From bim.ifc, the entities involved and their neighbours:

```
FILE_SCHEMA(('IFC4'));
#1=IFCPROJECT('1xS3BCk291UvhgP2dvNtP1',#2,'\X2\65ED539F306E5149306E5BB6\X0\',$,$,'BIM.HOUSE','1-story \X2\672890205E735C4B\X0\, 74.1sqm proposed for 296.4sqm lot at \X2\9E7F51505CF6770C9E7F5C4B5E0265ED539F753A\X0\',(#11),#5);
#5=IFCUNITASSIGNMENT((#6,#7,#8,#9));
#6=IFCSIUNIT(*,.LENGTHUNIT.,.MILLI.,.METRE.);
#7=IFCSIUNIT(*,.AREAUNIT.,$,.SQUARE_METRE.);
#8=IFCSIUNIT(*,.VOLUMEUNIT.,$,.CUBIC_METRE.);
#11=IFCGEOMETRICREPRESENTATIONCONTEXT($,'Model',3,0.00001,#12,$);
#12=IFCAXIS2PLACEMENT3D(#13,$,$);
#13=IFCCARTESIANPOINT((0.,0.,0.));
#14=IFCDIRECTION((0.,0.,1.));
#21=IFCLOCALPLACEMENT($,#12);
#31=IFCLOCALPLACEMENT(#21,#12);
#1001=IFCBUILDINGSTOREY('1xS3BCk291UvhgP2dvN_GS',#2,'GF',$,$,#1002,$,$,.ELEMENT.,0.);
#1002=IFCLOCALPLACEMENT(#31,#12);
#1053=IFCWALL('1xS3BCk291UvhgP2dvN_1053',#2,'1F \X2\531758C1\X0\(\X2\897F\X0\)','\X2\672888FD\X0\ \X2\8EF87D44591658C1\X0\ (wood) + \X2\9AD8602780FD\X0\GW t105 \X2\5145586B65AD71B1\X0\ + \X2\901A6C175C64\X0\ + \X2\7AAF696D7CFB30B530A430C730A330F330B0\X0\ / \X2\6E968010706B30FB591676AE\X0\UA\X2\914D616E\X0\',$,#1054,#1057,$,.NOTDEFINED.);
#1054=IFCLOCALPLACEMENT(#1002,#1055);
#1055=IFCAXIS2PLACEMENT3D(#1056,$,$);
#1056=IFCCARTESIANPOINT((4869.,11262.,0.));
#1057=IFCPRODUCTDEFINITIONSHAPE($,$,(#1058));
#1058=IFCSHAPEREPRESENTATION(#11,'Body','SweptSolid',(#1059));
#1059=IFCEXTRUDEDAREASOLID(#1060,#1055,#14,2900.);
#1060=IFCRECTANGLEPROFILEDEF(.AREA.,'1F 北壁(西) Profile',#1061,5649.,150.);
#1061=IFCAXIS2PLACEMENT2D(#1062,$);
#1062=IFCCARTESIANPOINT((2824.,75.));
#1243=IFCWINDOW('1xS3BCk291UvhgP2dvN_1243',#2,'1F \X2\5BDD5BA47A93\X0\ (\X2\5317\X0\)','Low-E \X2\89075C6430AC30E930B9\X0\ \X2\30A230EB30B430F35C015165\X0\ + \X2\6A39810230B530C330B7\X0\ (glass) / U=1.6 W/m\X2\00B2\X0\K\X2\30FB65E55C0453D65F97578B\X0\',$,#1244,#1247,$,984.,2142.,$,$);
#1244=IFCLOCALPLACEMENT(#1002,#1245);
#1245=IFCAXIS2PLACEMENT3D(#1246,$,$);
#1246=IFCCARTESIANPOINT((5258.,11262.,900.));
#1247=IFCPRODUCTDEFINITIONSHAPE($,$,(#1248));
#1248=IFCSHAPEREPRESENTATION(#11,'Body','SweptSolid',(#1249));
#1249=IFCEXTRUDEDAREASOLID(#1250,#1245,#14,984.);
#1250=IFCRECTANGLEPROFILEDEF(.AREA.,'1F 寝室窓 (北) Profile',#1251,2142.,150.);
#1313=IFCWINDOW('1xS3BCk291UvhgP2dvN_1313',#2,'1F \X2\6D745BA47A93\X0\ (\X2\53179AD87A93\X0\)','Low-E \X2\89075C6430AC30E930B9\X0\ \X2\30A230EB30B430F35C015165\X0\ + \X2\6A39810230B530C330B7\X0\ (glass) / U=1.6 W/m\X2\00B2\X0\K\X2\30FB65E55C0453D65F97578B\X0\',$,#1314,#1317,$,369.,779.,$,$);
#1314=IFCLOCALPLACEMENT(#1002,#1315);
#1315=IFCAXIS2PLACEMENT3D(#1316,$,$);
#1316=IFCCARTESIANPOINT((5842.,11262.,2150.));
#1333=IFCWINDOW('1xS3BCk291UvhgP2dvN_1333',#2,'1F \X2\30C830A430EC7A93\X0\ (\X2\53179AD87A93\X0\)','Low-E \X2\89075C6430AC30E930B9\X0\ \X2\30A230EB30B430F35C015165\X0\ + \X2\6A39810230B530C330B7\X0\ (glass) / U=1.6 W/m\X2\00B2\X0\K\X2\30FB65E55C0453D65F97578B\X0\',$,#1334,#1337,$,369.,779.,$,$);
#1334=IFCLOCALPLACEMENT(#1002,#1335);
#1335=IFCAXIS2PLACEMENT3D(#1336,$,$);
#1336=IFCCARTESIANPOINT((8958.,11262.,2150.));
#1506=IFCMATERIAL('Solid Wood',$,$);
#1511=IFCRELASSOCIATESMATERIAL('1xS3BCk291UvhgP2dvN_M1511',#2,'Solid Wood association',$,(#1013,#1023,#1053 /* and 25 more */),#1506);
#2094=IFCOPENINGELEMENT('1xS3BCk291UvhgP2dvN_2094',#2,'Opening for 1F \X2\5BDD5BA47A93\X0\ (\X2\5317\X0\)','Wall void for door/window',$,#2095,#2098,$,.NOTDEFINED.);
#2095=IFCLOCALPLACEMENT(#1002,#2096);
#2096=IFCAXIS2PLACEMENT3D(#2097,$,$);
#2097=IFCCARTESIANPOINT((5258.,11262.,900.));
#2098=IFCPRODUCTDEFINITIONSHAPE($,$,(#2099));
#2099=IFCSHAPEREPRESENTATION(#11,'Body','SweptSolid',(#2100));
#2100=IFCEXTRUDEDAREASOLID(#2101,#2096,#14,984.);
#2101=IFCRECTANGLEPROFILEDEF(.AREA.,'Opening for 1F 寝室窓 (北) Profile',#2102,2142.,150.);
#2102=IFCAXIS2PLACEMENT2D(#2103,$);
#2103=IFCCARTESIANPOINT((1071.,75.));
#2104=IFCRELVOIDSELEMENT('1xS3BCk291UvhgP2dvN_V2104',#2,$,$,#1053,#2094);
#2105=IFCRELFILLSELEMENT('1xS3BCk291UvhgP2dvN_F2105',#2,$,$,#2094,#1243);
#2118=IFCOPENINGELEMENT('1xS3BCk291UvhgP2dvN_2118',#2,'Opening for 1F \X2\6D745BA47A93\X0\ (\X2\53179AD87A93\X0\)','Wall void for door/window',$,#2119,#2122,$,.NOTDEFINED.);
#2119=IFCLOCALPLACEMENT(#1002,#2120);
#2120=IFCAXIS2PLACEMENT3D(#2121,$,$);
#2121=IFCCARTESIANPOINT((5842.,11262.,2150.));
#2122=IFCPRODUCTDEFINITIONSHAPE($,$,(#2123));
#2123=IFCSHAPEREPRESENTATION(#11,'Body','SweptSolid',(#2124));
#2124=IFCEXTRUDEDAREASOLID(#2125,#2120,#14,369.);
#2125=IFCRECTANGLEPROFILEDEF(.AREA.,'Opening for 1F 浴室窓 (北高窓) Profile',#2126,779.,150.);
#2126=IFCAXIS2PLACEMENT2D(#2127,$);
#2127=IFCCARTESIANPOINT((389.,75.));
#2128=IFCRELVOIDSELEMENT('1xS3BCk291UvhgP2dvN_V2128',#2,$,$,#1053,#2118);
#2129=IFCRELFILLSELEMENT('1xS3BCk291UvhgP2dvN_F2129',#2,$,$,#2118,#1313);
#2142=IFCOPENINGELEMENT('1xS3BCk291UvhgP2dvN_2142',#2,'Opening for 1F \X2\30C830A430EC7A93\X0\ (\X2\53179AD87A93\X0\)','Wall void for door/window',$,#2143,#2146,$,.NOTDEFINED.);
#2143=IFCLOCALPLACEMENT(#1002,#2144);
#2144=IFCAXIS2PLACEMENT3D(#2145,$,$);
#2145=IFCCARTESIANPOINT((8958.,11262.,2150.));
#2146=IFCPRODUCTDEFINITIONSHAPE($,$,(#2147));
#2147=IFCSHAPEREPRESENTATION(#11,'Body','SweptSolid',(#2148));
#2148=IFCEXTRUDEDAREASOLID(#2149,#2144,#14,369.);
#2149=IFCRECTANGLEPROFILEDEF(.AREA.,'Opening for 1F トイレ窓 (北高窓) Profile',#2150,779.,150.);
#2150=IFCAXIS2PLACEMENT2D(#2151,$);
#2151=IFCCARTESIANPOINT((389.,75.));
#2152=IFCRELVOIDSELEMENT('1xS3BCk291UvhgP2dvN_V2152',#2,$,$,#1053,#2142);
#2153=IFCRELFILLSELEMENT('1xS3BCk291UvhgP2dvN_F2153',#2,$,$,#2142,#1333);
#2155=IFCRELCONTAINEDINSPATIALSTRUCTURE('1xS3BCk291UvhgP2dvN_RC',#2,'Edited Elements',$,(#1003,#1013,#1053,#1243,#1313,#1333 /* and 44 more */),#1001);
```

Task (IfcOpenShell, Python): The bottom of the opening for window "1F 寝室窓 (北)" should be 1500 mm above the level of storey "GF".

```python
import numpy as np
import ifcopenshell
import ifcopenshell.api.geometry
import ifcopenshell.geom
import ifcopenshell.util.element
import ifcopenshell.util.placement
import ifcopenshell.util.shape
import ifcopenshell.util.unit

model = ifcopenshell.open("bim.ifc")
unit_scale = ifcopenshell.util.unit.calculate_unit_scale(model)

window = model.by_guid("1xS3BCk291UvhgP2dvN_1243")
opening = window.FillsVoids[0].RelatingOpeningElement
storey = ifcopenshell.util.element.get_container(window, ifc_class="IfcBuildingStorey")
level = ifcopenshell.util.placement.get_local_placement(storey.ObjectPlacement)[2, 3]

# The opening's origin need not be at the sill, so measure its lowest point.
shape = ifcopenshell.geom.create_shape(ifcopenshell.geom.settings(), opening)
bottom = ifcopenshell.util.shape.get_shape_bottom_elevation(shape, shape.geometry) / unit_scale
dz = level + 1500.0 - bottom

shift = np.array([0.0, 0.0, dz])
# The window is not placed relative to its opening, so move both.
for product in (opening, window):
    matrix = ifcopenshell.util.placement.get_local_placement(product.ObjectPlacement)
    matrix[:3, 3] += shift
    ifcopenshell.api.geometry.edit_object_placement(model, product=product, matrix=matrix, is_si=False)

print(f"moved by {dz * unit_scale:+.3f} m")

model.write("bim-out.ifc")
```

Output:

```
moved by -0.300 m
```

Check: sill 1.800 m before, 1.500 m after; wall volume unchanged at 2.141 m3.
